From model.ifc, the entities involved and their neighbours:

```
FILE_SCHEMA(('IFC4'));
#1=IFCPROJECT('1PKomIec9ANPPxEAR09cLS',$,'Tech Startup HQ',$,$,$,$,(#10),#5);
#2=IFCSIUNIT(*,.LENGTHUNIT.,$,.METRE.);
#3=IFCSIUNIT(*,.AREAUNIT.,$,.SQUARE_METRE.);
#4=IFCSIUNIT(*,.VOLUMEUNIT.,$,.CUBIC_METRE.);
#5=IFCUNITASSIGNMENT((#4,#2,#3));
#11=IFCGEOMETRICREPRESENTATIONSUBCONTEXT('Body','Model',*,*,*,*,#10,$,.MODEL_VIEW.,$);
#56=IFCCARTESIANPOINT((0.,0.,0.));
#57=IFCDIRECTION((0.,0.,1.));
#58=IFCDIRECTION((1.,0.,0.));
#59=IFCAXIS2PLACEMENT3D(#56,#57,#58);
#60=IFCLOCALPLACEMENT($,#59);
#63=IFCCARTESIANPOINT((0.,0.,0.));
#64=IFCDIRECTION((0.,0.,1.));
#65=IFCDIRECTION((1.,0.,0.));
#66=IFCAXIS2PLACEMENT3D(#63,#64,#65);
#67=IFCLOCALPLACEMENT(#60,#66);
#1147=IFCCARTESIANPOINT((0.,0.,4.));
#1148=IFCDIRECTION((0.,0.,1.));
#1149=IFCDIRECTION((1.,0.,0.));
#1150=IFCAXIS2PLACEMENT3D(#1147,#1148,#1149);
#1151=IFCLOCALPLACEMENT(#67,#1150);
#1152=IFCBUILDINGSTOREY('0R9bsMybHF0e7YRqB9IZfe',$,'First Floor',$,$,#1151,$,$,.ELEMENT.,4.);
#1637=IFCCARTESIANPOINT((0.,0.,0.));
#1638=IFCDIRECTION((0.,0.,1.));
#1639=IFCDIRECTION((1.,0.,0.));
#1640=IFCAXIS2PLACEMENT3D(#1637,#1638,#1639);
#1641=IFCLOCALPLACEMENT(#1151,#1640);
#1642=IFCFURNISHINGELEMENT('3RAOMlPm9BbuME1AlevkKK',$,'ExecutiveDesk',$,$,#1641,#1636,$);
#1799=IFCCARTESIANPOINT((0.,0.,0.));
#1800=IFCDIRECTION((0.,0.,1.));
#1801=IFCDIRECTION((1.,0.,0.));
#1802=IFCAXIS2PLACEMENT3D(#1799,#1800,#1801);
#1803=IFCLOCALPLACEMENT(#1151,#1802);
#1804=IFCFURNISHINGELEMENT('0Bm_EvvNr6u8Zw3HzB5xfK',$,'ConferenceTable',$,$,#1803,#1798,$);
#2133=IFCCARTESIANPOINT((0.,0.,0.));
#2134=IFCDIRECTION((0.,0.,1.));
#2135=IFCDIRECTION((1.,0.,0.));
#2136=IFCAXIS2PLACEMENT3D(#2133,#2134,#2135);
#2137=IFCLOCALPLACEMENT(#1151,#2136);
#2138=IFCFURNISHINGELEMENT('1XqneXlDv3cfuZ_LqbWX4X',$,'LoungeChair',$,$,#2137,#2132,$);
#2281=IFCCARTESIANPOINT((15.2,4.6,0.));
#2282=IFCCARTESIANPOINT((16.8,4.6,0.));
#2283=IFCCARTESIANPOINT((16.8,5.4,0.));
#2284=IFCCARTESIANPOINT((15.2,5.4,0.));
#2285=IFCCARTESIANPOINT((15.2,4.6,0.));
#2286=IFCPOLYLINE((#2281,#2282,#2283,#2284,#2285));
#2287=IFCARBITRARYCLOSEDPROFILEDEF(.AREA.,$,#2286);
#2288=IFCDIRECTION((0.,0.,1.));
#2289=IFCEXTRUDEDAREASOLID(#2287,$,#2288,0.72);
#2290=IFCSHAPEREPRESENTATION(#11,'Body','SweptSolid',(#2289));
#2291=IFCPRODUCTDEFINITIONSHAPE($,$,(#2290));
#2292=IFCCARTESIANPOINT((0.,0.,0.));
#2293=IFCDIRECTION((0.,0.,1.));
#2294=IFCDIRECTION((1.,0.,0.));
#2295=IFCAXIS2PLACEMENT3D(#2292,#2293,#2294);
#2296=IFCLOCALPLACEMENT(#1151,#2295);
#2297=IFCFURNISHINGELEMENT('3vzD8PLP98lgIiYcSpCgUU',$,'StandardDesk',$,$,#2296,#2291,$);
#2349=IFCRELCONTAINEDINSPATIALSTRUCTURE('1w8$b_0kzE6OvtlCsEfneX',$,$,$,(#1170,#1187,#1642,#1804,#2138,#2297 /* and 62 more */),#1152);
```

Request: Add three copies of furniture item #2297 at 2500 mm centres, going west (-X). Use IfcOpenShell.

```python
import numpy as np
import ifcopenshell
import ifcopenshell.api.geometry
import ifcopenshell.api.root
import ifcopenshell.util.element
import ifcopenshell.util.placement

model = ifcopenshell.open("model.ifc")

source = model.by_id(2297)
base = ifcopenshell.util.placement.get_local_placement(source.ObjectPlacement)
step = np.array([-1.0, 0.0, 0.0]) * 2.5

for i in range(1, 4):
    copy = ifcopenshell.api.root.copy_class(model, product=source)
    copy.Representation = ifcopenshell.util.element.copy_deep(
        model, source.Representation, exclude=["IfcGeometricRepresentationContext", "IfcRepresentationMap"]
    )
    matrix = base.copy()
    matrix[:3, 3] += i * step
    print("added at", matrix[:3, 3].round(3) + 0.0)
    ifcopenshell.api.geometry.edit_object_placement(model, product=copy, matrix=matrix, is_si=False)

model.write("model_rev.ifc")
```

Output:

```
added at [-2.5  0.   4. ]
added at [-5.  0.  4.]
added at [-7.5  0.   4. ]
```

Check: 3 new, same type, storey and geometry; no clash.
